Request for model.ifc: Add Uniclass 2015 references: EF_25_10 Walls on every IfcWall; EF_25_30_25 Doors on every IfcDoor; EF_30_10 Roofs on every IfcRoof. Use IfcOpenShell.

First a look at what the model holds.

```python
import ifcopenshell

model = ifcopenshell.open("model.ifc")
print(model.schema)
print("classifications:", [c.Name for c in model.by_type("IfcClassification")])
for ifc_class in ("IfcDoor", "IfcRoof", "IfcStair", "IfcWall", "IfcWindow"):
    print(ifc_class, len(model.by_type(ifc_class)))
```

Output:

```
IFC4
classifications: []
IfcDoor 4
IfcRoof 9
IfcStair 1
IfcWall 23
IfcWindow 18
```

```python
import ifcopenshell
import ifcopenshell.api.classification

model = ifcopenshell.open("model.ifc")

system = ifcopenshell.api.classification.add_classification(model, classification="Uniclass 2015")

codes = {
    "IfcWall": ("EF_25_10", "Walls"),
    "IfcDoor": ("EF_25_30_25", "Doors"),
    "IfcRoof": ("EF_30_10", "Roofs"),
}
for ifc_class, (code, name) in codes.items():
    products = model.by_type(ifc_class)
    ifcopenshell.api.classification.add_reference(
        model, products=products, classification=system, identification=code, name=name
    )
    print(code, len(products))

model.write("model_v2.ifc")
```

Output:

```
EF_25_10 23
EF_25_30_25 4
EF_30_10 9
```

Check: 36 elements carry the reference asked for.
